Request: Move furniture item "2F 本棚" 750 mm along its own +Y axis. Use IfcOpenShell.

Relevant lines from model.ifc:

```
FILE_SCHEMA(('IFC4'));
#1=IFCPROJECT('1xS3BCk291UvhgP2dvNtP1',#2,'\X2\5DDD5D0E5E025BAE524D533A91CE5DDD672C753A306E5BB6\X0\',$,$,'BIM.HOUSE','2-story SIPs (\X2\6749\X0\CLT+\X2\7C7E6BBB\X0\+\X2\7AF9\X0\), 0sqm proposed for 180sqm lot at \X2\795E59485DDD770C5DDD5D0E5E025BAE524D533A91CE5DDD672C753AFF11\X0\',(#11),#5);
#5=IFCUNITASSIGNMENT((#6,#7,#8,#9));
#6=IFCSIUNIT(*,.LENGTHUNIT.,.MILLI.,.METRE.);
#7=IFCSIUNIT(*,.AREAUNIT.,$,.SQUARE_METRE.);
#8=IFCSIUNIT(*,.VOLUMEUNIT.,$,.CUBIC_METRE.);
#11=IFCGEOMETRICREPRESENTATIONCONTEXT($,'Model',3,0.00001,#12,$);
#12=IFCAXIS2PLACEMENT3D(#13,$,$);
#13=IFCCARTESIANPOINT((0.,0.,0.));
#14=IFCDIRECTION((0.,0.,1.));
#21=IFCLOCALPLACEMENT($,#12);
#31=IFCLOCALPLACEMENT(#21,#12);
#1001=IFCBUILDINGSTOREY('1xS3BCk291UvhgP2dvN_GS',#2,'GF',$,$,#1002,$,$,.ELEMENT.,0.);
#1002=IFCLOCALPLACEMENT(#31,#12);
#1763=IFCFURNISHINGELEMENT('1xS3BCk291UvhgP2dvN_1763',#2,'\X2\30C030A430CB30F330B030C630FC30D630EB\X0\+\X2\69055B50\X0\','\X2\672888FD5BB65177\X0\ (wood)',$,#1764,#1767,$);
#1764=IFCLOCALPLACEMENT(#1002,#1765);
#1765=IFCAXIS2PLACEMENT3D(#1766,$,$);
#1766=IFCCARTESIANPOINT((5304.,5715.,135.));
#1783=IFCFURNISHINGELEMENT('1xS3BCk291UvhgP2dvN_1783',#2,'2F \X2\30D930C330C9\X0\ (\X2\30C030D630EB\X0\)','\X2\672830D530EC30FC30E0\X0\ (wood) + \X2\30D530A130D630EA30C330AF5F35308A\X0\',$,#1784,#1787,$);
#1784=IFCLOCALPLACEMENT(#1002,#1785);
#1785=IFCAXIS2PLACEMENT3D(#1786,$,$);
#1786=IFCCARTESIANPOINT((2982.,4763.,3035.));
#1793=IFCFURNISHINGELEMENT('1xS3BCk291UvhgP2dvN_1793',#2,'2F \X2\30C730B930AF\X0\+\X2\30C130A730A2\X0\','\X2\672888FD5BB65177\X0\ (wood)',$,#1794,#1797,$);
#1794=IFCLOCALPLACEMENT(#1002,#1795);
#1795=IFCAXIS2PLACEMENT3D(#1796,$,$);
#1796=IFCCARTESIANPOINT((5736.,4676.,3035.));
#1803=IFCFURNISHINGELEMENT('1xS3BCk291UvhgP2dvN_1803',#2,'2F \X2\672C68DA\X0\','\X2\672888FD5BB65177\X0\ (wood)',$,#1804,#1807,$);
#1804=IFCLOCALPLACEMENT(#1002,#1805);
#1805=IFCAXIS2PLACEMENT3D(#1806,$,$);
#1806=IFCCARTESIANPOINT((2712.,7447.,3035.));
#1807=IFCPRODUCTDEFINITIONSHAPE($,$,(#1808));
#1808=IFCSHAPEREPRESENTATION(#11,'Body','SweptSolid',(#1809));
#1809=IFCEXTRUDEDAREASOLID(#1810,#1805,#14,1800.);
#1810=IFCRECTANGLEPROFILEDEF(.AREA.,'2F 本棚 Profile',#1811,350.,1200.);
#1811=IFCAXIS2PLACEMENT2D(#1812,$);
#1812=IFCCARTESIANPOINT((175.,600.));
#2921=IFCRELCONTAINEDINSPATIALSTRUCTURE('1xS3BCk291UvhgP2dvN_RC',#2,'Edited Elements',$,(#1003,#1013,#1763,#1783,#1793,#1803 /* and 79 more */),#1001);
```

```python
import ifcopenshell
import ifcopenshell.api.geometry
import ifcopenshell.util.placement
import ifcopenshell.util.unit

model = ifcopenshell.open("model.ifc")
unit_scale = ifcopenshell.util.unit.calculate_unit_scale(model)

item = model.by_id(1803)
matrix = ifcopenshell.util.placement.get_local_placement(item.ObjectPlacement)
matrix[:3, 3] += matrix[:3, 1] * 0.75 / unit_scale
ifcopenshell.api.geometry.edit_object_placement(model, product=item, matrix=matrix, is_si=False)

print(ifcopenshell.util.placement.get_local_placement(item.ObjectPlacement).round(3) + 0.0)

model.write("model_edited.ifc")
```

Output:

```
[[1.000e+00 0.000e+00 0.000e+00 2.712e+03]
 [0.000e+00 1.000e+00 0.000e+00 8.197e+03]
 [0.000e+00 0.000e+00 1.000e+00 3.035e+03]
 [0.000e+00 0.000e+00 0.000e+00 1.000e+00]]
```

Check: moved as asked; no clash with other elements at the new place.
